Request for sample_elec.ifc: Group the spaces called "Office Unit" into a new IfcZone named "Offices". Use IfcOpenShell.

First a look at what the model holds.

```python
import ifcopenshell

model = ifcopenshell.open("sample_elec.ifc")
print(model.schema)
seen = {}
for space in model.by_type("IfcSpace"):
    seen[space.LongName] = seen.get(space.LongName, 0) + 1
for name, count in sorted(seen.items(), key=str):
    print(count, "x", name)
print("zones:", [z.Name for z in model.by_type("IfcZone")][:20])
```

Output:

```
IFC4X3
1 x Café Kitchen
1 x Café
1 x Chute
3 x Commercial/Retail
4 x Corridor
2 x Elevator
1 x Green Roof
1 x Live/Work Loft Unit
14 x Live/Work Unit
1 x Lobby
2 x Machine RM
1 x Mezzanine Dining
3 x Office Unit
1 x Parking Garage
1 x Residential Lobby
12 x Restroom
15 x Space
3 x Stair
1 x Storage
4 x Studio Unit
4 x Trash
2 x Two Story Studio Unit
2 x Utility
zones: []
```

```python
import ifcopenshell
import ifcopenshell.api.group
import ifcopenshell.api.root

model = ifcopenshell.open("sample_elec.ifc")

names = {"Office Unit"}
spaces = [s for s in model.by_type("IfcSpace") if s.LongName in names]

zone = ifcopenshell.api.root.create_entity(model, ifc_class="IfcZone", name="Offices")
ifcopenshell.api.group.assign_group(model, products=spaces, group=zone)
print(len(spaces), "spaces in", zone.Name)

model.write("sample_elec_v2.ifc")
```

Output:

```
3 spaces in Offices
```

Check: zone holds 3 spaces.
